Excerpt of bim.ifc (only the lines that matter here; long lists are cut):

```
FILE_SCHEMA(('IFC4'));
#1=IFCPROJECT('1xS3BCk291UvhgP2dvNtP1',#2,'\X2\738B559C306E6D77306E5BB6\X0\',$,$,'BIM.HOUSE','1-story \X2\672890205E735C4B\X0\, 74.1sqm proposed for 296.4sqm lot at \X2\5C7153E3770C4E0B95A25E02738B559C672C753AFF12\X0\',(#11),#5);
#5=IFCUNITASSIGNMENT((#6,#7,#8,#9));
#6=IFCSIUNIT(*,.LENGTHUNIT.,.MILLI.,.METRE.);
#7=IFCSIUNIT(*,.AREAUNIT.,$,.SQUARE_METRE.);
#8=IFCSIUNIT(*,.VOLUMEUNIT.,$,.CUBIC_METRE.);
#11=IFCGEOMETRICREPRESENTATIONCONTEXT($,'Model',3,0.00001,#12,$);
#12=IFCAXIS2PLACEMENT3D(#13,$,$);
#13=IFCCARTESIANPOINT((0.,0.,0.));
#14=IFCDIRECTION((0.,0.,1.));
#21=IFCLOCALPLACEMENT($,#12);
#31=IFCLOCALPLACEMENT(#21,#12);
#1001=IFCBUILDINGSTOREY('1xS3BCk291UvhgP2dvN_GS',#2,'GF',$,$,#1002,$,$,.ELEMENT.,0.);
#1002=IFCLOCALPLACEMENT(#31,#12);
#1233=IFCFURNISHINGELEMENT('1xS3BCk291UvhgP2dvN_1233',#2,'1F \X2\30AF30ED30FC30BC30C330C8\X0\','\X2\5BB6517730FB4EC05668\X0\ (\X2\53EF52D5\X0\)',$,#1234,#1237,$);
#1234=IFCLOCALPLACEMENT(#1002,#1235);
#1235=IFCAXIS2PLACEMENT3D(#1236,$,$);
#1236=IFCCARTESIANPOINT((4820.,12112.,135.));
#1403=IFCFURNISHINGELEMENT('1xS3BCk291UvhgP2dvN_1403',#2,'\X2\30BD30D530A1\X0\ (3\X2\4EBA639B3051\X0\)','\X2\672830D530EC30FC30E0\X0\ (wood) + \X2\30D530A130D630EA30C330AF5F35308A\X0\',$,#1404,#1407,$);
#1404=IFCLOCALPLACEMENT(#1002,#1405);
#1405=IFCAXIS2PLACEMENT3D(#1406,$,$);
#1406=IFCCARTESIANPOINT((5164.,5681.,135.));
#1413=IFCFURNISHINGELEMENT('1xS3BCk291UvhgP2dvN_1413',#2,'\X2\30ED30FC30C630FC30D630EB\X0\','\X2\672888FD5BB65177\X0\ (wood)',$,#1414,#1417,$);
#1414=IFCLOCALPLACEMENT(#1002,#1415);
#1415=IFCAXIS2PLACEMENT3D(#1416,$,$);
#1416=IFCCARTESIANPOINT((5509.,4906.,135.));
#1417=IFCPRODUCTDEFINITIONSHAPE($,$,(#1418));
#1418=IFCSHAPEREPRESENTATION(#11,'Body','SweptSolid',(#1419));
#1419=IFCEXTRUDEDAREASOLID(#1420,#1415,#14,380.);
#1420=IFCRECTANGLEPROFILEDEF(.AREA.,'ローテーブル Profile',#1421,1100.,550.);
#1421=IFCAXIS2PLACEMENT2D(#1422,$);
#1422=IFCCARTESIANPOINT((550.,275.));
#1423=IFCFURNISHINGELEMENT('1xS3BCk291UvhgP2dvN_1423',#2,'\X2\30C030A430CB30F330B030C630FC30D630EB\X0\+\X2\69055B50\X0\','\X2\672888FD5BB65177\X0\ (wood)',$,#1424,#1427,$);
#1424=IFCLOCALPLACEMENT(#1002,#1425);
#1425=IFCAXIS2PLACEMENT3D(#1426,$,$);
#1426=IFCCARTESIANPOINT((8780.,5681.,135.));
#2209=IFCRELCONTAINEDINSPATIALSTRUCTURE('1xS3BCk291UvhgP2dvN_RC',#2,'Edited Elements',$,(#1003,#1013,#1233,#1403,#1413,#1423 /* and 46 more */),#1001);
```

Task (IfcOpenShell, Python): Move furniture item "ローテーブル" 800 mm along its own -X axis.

```python
import ifcopenshell
import ifcopenshell.api.geometry
import ifcopenshell.util.placement

model = ifcopenshell.open("bim.ifc")

item = model.by_guid("1xS3BCk291UvhgP2dvN_1413")
matrix = ifcopenshell.util.placement.get_local_placement(item.ObjectPlacement)
matrix[:3, 3] -= matrix[:3, 0] * 800.0
ifcopenshell.api.geometry.edit_object_placement(model, product=item, matrix=matrix, is_si=False)

print(ifcopenshell.util.placement.get_local_placement(item.ObjectPlacement).round(3) + 0.0)

model.write("bim_v2.ifc")
```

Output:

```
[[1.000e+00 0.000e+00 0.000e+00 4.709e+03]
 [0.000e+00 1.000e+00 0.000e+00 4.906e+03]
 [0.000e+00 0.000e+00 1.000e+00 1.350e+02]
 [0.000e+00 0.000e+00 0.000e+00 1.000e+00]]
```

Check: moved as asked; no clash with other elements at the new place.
